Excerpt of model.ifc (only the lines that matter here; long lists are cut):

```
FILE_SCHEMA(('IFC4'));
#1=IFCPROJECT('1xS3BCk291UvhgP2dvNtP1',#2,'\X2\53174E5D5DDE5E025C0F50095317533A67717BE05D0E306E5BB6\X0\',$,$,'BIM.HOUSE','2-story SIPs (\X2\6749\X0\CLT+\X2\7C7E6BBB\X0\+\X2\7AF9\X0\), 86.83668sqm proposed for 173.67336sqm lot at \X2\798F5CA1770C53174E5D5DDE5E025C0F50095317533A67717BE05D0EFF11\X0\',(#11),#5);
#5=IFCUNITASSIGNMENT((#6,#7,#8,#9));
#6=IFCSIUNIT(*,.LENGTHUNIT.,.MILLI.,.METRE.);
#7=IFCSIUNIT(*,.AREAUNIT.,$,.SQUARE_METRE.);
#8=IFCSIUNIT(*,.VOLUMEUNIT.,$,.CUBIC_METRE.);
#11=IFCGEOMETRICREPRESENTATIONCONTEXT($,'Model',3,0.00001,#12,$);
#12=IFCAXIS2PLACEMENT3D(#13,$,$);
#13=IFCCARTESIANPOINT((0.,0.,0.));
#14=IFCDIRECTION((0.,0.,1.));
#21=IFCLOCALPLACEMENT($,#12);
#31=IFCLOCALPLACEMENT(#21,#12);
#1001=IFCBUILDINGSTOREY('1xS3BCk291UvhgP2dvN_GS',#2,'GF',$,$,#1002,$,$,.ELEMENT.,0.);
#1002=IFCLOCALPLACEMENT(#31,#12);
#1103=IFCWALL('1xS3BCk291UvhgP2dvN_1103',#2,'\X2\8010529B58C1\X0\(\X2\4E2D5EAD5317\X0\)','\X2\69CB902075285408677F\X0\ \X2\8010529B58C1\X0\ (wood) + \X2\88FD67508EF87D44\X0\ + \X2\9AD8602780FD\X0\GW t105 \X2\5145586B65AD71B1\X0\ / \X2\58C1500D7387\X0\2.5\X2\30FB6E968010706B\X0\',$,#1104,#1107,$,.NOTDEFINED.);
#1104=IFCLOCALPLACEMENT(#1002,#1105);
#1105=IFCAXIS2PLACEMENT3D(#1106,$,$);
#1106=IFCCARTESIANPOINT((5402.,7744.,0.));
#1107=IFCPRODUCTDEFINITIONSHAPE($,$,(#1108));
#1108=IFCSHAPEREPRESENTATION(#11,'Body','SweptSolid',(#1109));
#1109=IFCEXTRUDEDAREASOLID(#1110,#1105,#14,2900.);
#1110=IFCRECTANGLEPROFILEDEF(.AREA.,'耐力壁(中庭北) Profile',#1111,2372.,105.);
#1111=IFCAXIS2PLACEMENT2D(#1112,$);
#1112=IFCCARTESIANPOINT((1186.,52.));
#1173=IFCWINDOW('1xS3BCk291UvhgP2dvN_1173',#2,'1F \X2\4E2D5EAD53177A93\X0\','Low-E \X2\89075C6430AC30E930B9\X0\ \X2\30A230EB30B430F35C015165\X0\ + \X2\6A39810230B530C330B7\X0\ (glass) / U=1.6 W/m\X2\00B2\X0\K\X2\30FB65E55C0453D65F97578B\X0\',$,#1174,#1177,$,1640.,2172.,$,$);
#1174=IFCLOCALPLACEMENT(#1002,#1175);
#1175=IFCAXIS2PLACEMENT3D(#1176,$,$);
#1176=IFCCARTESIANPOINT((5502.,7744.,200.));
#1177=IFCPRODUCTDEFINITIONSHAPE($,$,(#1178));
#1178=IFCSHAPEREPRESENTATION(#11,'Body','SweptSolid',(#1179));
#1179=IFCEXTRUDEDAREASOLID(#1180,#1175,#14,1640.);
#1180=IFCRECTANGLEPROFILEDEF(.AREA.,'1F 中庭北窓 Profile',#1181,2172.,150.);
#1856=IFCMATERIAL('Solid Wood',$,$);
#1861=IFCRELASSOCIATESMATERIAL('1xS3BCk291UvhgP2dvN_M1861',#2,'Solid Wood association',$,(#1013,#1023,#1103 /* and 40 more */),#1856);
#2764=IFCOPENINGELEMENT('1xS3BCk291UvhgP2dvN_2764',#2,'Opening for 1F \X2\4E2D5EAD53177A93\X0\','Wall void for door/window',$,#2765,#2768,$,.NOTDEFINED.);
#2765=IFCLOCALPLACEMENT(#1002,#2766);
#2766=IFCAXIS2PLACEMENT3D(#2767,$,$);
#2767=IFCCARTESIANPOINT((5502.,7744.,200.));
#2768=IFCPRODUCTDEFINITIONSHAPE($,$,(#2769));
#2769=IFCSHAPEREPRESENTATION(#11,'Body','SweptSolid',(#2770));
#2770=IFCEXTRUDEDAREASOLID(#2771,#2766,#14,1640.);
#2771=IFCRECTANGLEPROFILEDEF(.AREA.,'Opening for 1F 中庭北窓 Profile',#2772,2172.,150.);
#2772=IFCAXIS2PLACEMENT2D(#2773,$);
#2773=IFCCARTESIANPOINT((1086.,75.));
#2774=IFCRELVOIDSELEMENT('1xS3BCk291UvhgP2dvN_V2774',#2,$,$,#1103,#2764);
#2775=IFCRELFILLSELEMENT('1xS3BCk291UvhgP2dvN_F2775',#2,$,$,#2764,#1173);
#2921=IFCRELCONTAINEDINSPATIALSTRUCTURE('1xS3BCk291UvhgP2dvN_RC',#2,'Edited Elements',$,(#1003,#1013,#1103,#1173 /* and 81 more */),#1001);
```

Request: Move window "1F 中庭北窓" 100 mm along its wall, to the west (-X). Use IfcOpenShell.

```python
import ifcopenshell
import ifcopenshell.api.geometry
import ifcopenshell.util.placement
import ifcopenshell.util.unit

model = ifcopenshell.open("model.ifc")
unit_scale = ifcopenshell.util.unit.calculate_unit_scale(model)

window = model.by_guid("1xS3BCk291UvhgP2dvN_1173")
opening = window.FillsVoids[0].RelatingOpeningElement
wall = opening.VoidsElements[0].RelatingBuildingElement

wall_matrix = ifcopenshell.util.placement.get_local_placement(wall.ObjectPlacement)
shift = wall_matrix[:3, 0] * -0.1 / unit_scale
before = ifcopenshell.util.placement.get_local_placement(window.ObjectPlacement)[:3, 3].copy()

# The window is not placed relative to its opening, so move both.
for product in (opening, window):
    matrix = ifcopenshell.util.placement.get_local_placement(product.ObjectPlacement)
    matrix[:3, 3] += shift
    ifcopenshell.api.geometry.edit_object_placement(model, product=product, matrix=matrix, is_si=False)

after = ifcopenshell.util.placement.get_local_placement(window.ObjectPlacement)[:3, 3]
print("window moved by", (after - before).round(3) + 0.0)

model.write("model-out.ifc")
```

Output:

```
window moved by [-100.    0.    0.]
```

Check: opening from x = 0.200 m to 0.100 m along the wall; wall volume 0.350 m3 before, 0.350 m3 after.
